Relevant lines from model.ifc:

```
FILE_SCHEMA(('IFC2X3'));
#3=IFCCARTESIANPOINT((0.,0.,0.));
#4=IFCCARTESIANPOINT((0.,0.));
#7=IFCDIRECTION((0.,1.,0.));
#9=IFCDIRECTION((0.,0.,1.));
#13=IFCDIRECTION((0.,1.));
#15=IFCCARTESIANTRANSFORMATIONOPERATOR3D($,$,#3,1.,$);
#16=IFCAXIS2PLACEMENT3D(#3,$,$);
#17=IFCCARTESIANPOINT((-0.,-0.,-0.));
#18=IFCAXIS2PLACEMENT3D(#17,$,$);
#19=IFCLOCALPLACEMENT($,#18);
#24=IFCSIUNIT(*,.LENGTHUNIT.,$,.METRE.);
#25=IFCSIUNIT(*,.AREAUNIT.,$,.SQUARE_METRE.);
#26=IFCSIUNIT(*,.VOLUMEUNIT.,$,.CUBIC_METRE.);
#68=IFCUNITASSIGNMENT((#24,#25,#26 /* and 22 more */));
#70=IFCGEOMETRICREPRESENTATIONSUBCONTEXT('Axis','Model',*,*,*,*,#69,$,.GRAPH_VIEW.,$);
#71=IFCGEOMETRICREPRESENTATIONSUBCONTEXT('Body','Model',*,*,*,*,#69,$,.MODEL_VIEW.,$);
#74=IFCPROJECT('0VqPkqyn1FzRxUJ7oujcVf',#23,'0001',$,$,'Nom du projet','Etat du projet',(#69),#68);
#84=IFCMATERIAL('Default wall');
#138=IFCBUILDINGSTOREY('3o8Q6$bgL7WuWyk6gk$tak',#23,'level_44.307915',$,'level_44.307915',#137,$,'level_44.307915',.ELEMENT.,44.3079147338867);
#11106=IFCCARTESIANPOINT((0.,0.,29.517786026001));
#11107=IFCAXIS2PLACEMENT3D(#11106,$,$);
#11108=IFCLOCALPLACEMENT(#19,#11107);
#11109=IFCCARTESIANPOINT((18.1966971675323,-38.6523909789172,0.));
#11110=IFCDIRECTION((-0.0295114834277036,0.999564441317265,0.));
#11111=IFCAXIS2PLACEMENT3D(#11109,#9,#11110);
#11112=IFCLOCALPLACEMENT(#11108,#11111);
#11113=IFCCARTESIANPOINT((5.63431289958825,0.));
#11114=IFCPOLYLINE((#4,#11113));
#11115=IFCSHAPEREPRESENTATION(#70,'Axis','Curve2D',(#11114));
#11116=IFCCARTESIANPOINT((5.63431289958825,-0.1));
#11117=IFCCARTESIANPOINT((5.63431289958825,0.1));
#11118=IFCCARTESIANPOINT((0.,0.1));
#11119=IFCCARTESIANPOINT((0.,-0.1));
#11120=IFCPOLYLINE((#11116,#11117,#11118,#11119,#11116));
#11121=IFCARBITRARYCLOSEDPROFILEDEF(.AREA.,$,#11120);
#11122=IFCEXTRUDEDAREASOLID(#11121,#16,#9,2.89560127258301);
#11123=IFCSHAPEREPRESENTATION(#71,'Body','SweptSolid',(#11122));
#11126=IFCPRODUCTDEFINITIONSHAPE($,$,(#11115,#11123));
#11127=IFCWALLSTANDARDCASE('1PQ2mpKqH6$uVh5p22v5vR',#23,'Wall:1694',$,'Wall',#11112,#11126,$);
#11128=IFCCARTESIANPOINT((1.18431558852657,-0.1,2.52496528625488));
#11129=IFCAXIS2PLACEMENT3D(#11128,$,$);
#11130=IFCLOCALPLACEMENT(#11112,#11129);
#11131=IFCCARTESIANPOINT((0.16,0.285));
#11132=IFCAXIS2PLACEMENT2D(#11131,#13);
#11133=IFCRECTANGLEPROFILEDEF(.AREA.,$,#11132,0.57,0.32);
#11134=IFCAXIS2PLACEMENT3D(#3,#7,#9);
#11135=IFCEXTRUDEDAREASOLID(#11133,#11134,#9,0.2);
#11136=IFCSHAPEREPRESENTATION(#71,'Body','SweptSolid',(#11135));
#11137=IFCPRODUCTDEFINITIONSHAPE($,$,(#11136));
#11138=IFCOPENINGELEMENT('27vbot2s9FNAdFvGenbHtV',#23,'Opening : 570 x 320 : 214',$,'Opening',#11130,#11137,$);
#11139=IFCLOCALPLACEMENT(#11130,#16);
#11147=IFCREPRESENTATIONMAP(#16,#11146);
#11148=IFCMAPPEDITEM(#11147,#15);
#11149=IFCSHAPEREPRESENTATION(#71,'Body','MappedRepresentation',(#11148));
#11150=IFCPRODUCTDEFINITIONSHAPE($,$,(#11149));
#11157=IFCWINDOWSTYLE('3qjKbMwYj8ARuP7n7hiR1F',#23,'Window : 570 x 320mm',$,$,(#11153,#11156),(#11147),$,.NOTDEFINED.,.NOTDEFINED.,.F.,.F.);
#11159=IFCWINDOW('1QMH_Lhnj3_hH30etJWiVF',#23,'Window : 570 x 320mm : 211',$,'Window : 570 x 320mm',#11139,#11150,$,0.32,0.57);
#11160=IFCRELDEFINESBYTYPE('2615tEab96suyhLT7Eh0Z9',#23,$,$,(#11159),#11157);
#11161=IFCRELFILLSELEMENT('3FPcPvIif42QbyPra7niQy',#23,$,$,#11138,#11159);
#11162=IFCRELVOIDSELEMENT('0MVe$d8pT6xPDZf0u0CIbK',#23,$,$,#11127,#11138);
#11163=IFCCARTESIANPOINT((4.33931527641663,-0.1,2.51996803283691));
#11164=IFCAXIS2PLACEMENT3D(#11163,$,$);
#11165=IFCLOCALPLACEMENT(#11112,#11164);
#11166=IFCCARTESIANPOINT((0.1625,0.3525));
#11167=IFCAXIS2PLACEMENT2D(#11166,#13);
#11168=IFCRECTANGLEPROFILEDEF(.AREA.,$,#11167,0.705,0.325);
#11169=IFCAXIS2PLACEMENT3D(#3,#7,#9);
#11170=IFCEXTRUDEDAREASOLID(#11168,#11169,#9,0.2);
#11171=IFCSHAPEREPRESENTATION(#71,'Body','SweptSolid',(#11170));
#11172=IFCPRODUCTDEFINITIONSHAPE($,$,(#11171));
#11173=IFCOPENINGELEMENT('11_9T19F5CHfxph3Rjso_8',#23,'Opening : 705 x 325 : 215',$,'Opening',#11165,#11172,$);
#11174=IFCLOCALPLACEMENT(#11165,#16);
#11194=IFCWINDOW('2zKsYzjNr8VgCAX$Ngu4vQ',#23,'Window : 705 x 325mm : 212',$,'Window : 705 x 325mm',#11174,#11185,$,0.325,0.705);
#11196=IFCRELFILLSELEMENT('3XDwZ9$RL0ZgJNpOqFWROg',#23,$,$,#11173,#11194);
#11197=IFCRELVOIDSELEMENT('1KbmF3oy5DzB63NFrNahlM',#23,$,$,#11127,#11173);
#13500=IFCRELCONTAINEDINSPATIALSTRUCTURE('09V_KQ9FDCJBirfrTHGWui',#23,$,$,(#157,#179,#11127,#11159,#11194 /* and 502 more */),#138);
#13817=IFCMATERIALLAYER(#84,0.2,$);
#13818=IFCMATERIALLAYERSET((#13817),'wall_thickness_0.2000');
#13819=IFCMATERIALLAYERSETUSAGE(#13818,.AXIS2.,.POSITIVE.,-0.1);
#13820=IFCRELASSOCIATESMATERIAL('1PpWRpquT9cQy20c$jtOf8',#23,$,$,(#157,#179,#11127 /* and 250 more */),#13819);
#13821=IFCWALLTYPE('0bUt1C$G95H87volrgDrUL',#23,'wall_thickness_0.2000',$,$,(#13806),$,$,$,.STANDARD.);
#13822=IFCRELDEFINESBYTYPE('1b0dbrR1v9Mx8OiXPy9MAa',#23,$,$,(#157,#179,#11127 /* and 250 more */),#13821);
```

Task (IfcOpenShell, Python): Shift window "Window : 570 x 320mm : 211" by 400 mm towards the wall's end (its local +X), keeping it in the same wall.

```python
import ifcopenshell
import ifcopenshell.api.geometry
import ifcopenshell.util.placement

model = ifcopenshell.open("model.ifc")

window = model.by_id(11159)
opening = window.FillsVoids[0].RelatingOpeningElement
wall = opening.VoidsElements[0].RelatingBuildingElement

wall_matrix = ifcopenshell.util.placement.get_local_placement(wall.ObjectPlacement)
shift = wall_matrix[:3, 0] * 0.4
before = ifcopenshell.util.placement.get_local_placement(window.ObjectPlacement)[:3, 3].copy()

# The window is placed relative to its opening, so it follows when the opening moves.
matrix = ifcopenshell.util.placement.get_local_placement(opening.ObjectPlacement)
matrix[:3, 3] += shift
ifcopenshell.api.geometry.edit_object_placement(
    model, product=opening, matrix=matrix, is_si=False, should_transform_children=True
)

after = ifcopenshell.util.placement.get_local_placement(window.ObjectPlacement)[:3, 3]
print("window moved by", (after - before).round(3) + 0.0)

model.write("model_edited.ifc")
```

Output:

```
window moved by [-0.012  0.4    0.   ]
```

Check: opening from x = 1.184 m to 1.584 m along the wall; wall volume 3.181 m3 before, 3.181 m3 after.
